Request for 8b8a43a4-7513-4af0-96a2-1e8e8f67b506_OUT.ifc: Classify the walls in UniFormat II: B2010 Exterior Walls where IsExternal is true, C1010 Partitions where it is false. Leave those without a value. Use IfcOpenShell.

First a look at what the model holds.

```python
import ifcopenshell
import ifcopenshell.util.element

model = ifcopenshell.open("8b8a43a4-7513-4af0-96a2-1e8e8f67b506_OUT.ifc")
print(model.schema)
print("classifications:", [c.Name for c in model.by_type("IfcClassification")])
values = [ifcopenshell.util.element.get_pset(e, "Pset_WallCommon", "IsExternal") for e in model.by_type("IfcWall")]
for value in (True, False, None):
    print("IsExternal", value, values.count(value))
```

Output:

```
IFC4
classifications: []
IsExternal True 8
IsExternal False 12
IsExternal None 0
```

```python
import ifcopenshell
import ifcopenshell.api.classification
import ifcopenshell.util.element

model = ifcopenshell.open("8b8a43a4-7513-4af0-96a2-1e8e8f67b506_OUT.ifc")

system = ifcopenshell.api.classification.add_classification(model, classification="UniFormat II")

walls = model.by_type("IfcWall")
external = {e: ifcopenshell.util.element.get_pset(e, "Pset_WallCommon", "IsExternal") for e in walls}
for flag, code, name in ((True, "B2010", "Exterior Walls"), (False, "C1010", "Partitions")):
    products = [e for e in walls if external[e] is flag]
    ifcopenshell.api.classification.add_reference(
        model, products=products, classification=system, identification=code, name=name
    )
    print(code, len(products))

model.write("8b8a43a4-7513-4af0-96a2-1e8e8f67b506_OUT_v2.ifc")
```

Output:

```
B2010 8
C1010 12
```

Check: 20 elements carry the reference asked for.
